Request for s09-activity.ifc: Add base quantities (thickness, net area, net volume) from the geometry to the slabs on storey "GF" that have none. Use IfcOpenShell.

First a look at what the model holds.

```python
import ifcopenshell
import ifcopenshell.util.element
import ifcopenshell.util.unit

model = ifcopenshell.open("s09-activity.ifc")
print(model.schema)
for unit_type in ("LENGTHUNIT", "AREAUNIT", "VOLUMEUNIT"):
    print(unit_type, ifcopenshell.util.unit.calculate_unit_scale(model, unit_type))
storey = next(s for s in model.by_type("IfcBuildingStorey") if s.Name == "GF")
slabs = [e for e in ifcopenshell.util.element.get_decomposition(storey) if e.is_a("IfcSlab")]
for e in sorted(slabs, key=lambda e: e.id()):
    print(e.id(), e.is_a(), e.Name, list(ifcopenshell.util.element.get_psets(e, qtos_only=True)), sep=" | ")
```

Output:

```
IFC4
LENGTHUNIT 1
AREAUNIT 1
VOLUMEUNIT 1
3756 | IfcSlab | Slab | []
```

```python
import ifcopenshell
import ifcopenshell.api.pset
import ifcopenshell.geom
import ifcopenshell.util.element
import ifcopenshell.util.shape
import ifcopenshell.util.unit

model = ifcopenshell.open("s09-activity.ifc")
unit_scale = ifcopenshell.util.unit.calculate_unit_scale(model)
area_scale = ifcopenshell.util.unit.calculate_unit_scale(model, "AREAUNIT")
volume_scale = ifcopenshell.util.unit.calculate_unit_scale(model, "VOLUMEUNIT")
settings = ifcopenshell.geom.settings()

storey = next(s for s in model.by_type("IfcBuildingStorey") if s.Name == "GF")
slabs = [e for e in ifcopenshell.util.element.get_decomposition(storey) if e.is_a("IfcSlab")]

for e in sorted(slabs, key=lambda e: e.id()):
    if ifcopenshell.util.element.get_psets(e, qtos_only=True, should_inherit=False):
        continue
    # Geometry comes back in metres, in the element's own axes.
    shape = ifcopenshell.geom.create_shape(settings, e)
    values = {
        "Width": ifcopenshell.util.shape.get_z(shape.geometry) / unit_scale,
        "NetArea": ifcopenshell.util.shape.get_footprint_area(shape.geometry) / area_scale,
        "NetVolume": ifcopenshell.util.shape.get_volume(shape.geometry) / volume_scale,
    }
    qto = ifcopenshell.api.pset.add_qto(model, product=e, name="Qto_SlabBaseQuantities")
    ifcopenshell.api.pset.edit_qto(model, qto=qto, properties=values)
    print(e.id(), {k: round(v, 3) for k, v in values.items()})

model.write("s09-activity-out.ifc")
```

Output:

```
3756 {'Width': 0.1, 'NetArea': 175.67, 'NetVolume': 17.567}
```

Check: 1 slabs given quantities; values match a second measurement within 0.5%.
